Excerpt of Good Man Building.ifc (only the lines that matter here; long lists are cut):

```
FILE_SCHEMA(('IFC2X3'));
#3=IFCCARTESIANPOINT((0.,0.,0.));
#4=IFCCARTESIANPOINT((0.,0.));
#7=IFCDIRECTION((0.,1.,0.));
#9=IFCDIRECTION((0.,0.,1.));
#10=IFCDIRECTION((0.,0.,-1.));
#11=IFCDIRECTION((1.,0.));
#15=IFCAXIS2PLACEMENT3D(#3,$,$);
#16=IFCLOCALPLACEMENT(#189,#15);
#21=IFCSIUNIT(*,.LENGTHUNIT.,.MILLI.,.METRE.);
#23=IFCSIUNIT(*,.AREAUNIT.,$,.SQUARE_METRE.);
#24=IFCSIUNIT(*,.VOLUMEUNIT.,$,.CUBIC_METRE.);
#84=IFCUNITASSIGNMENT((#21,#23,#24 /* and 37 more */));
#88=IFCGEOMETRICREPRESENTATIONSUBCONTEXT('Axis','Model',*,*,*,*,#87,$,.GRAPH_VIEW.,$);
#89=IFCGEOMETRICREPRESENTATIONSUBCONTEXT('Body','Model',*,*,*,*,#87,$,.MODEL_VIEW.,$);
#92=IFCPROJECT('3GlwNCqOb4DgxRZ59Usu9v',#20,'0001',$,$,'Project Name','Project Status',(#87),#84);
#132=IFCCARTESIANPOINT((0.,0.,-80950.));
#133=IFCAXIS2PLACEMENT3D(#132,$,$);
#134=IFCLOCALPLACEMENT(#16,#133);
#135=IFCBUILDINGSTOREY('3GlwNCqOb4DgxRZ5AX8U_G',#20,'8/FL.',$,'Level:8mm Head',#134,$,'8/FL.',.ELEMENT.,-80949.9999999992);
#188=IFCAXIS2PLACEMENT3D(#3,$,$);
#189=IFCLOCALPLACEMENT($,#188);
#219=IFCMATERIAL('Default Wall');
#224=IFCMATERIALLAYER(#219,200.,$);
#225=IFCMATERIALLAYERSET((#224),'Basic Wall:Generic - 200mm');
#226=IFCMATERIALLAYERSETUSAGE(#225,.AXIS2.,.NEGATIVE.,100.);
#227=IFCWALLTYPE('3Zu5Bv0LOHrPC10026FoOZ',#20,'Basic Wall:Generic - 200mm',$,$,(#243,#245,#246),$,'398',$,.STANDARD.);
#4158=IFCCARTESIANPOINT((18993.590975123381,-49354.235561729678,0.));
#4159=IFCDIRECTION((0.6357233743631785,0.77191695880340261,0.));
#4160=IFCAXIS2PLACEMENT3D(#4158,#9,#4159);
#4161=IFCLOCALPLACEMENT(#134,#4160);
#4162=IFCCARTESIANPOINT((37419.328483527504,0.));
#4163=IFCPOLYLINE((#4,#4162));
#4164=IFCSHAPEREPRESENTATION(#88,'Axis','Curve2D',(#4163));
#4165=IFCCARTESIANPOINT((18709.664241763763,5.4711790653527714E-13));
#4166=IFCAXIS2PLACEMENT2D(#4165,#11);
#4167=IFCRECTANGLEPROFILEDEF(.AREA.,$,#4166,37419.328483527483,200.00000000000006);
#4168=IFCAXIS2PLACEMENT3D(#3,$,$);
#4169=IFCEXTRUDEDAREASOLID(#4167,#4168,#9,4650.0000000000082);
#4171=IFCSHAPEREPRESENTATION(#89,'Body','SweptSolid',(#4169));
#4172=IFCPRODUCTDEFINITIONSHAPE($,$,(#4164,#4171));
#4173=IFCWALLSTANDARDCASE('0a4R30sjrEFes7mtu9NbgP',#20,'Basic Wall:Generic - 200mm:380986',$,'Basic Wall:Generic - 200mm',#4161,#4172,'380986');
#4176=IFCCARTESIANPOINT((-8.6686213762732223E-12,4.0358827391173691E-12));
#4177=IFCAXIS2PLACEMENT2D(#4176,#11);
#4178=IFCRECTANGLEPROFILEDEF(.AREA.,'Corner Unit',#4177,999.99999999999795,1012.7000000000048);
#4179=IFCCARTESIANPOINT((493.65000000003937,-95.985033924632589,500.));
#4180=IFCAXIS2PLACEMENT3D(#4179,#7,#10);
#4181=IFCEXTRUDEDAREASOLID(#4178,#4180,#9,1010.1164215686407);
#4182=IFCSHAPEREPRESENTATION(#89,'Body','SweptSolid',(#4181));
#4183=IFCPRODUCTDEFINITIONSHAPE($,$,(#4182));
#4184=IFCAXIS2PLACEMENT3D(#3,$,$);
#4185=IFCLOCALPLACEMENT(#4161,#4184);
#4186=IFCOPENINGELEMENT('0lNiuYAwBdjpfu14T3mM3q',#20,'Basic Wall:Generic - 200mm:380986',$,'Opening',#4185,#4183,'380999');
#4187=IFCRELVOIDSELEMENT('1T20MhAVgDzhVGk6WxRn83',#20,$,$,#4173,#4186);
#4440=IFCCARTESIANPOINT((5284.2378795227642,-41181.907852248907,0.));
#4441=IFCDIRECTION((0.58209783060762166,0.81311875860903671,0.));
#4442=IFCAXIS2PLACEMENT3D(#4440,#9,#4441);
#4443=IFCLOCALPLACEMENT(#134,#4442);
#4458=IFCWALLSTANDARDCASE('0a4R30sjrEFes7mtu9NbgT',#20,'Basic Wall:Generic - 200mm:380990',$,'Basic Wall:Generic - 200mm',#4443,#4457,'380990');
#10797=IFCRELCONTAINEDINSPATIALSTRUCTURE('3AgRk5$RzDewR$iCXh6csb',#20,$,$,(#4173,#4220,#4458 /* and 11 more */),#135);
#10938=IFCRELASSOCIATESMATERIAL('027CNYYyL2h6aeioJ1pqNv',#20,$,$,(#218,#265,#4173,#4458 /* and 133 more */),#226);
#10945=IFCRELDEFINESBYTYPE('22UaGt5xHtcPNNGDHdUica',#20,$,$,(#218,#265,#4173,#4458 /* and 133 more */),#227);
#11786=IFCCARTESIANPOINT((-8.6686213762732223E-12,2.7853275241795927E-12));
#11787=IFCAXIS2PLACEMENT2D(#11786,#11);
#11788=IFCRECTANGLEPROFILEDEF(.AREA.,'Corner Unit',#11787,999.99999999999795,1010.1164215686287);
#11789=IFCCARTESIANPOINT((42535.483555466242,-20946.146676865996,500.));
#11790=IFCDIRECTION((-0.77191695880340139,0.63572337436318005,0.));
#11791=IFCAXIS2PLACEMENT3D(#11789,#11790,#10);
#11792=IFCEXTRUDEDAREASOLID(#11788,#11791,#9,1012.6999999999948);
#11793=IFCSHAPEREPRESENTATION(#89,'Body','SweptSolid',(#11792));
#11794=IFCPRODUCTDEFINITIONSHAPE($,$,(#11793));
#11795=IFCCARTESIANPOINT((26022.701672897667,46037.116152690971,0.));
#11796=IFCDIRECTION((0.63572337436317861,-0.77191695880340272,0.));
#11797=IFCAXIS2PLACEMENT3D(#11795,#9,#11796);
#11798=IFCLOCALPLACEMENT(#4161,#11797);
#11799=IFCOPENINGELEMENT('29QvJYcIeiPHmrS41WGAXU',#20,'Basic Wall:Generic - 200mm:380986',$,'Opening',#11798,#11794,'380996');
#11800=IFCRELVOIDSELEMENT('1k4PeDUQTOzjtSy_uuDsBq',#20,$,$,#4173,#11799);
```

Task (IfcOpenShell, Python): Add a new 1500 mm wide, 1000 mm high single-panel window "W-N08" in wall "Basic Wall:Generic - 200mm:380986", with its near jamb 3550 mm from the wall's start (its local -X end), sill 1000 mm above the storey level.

```python
import numpy as np
import ifcopenshell
import ifcopenshell.api.feature
import ifcopenshell.api.geometry
import ifcopenshell.api.root
import ifcopenshell.api.spatial
import ifcopenshell.api.type
import ifcopenshell.geom
import ifcopenshell.util.element
import ifcopenshell.util.placement
import ifcopenshell.util.representation
import ifcopenshell.util.shape
import ifcopenshell.util.unit

model = ifcopenshell.open("Good Man Building.ifc")
unit_scale = ifcopenshell.util.unit.calculate_unit_scale(model)
settings = ifcopenshell.geom.settings()


def volume(element):
    """Net volume in cubic metres, openings subtracted."""
    shape = ifcopenshell.geom.create_shape(settings, element)
    return ifcopenshell.util.shape.get_volume(shape.geometry)


wall = model.by_guid("0a4R30sjrEFes7mtu9NbgP")
storey = ifcopenshell.util.element.get_container(wall, ifc_class="IfcBuildingStorey")
context = ifcopenshell.util.representation.get_context(model, "Model", "Body", "MODEL_VIEW")
before = volume(wall)

width, height, from_end, sill = 1.5, 1, 3.55, 1  # metres

# The wall runs along its own X axis, and the end named is its -X end.
wall_shape = ifcopenshell.geom.create_shape(settings, wall)
x, y, z = ifcopenshell.util.shape.get_vertices(wall_shape.geometry).T
start = x.min() + from_end
face, thickness = float(y.min()), float(y.max() - y.min())
wall_matrix = ifcopenshell.util.placement.get_local_placement(wall.ObjectPlacement)
level = ifcopenshell.util.placement.get_local_placement(storey.ObjectPlacement)[2, 3]


def in_wall(x, y):
    """Placement at x, y metres in the wall's axes, at sill height."""
    matrix = wall_matrix.copy()
    matrix[:, 3] = wall_matrix @ np.array([x / unit_scale, y / unit_scale, 0.0, 1.0])
    matrix[2, 3] = level + sill / unit_scale
    return matrix


# Opening: a box that overshoots both wall faces by 50 mm.
opening = ifcopenshell.api.root.create_entity(model, ifc_class="IfcOpeningElement")
box = ifcopenshell.api.geometry.add_wall_representation(
    model, context=context, length=width, height=height, thickness=thickness + 0.1
)
ifcopenshell.api.geometry.assign_representation(model, product=opening, representation=box)
ifcopenshell.api.geometry.edit_object_placement(model, product=opening, matrix=in_wall(start, face - 0.05), is_si=False)
ifcopenshell.api.feature.add_feature(model, feature=opening, element=wall)

window = ifcopenshell.api.root.create_entity(model, ifc_class="IfcWindow", name="W-N08")
window.OverallWidth, window.OverallHeight = width / unit_scale, height / unit_scale
body = ifcopenshell.api.geometry.add_window_representation(
    model,
    context=context,
    overall_width=window.OverallWidth,
    overall_height=window.OverallHeight,
    partition_type="SINGLE_PANEL",
)
ifcopenshell.api.geometry.assign_representation(model, product=window, representation=body)
ifcopenshell.api.spatial.assign_container(model, products=[window], relating_structure=storey)
fills = ifcopenshell.api.feature.add_filling(model, opening=opening, element=window)
fills.OwnerHistory = window.OwnerHistory  # required in IFC2X3

# IFC2X3 keeps the operation on the window style.
style = ifcopenshell.api.root.create_entity(model, ifc_class="IfcWindowStyle", name="W-N08")
style.OperationType, style.ConstructionType = "SINGLE_PANEL", "NOTDEFINED"
style.ParameterTakesPrecedence = style.Sizeable = False
ifcopenshell.api.type.assign_type(model, related_objects=[window], relating_type=style)

# Centre the window in the wall's thickness.
ifcopenshell.api.geometry.edit_object_placement(model, product=window, matrix=in_wall(start, face), is_si=False)
window_shape = ifcopenshell.geom.create_shape(settings, window)
depth = ifcopenshell.util.shape.get_vertices(window_shape.geometry)[:, 1]
offset = face + thickness / 2 - (depth.min() + depth.max()) / 2
ifcopenshell.api.geometry.edit_object_placement(model, product=window, matrix=in_wall(start, offset), is_si=False)

after = volume(wall)

print(f"wall volume {before:.3f} -> {after:.3f} m3")

model.write("Good Man Building_v2.ifc")
```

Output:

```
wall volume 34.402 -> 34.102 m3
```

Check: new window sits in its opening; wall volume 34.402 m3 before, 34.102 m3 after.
